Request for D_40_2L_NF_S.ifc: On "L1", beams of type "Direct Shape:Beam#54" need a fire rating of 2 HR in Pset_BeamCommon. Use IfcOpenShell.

First a look at what the model holds.

```python
import ifcopenshell
import ifcopenshell.util.element

model = ifcopenshell.open("D_40_2L_NF_S.ifc")
print(model.schema)
storey = next(s for s in model.by_type("IfcBuildingStorey") if s.Name == "L1")
beams = [e for e in ifcopenshell.util.element.get_decomposition(storey) if e.is_a("IfcBeam")]
seen = {}
for e in beams:
    element_type = ifcopenshell.util.element.get_type(e)
    key = (element_type.Name if element_type != e and element_type else None, ifcopenshell.util.element.get_pset(e, "Pset_BeamCommon", "FireRating"))
    seen[key] = seen.get(key, 0) + 1
for (name, value), count in sorted(seen.items(), key=str):
    print(count, "x", name, "|", value)
```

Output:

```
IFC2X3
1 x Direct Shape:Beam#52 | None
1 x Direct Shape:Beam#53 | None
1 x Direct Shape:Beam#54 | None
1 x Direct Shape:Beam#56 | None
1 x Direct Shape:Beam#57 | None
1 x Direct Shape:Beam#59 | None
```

```python
import ifcopenshell
import ifcopenshell.api.pset
import ifcopenshell.util.element

model = ifcopenshell.open("D_40_2L_NF_S.ifc")

storey = next(s for s in model.by_type("IfcBuildingStorey") if s.Name == "L1")
beams = [e for e in ifcopenshell.util.element.get_decomposition(storey) if e.is_a("IfcBeam")]

count = 0
for e in beams:
    element_type = ifcopenshell.util.element.get_type(e)
    if element_type in (None, e) or element_type.Name != "Direct Shape:Beam#54":
        continue
    # add_pset returns the element's existing set when there is one.
    pset = ifcopenshell.api.pset.add_pset(model, product=e, name="Pset_BeamCommon")
    ifcopenshell.api.pset.edit_pset(model, pset=pset, properties={"FireRating": "2 HR"})
    count += 1

print(count, "beams updated")

model.write("D_40_2L_NF_S_edited.ifc")
```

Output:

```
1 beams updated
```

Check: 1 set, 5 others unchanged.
